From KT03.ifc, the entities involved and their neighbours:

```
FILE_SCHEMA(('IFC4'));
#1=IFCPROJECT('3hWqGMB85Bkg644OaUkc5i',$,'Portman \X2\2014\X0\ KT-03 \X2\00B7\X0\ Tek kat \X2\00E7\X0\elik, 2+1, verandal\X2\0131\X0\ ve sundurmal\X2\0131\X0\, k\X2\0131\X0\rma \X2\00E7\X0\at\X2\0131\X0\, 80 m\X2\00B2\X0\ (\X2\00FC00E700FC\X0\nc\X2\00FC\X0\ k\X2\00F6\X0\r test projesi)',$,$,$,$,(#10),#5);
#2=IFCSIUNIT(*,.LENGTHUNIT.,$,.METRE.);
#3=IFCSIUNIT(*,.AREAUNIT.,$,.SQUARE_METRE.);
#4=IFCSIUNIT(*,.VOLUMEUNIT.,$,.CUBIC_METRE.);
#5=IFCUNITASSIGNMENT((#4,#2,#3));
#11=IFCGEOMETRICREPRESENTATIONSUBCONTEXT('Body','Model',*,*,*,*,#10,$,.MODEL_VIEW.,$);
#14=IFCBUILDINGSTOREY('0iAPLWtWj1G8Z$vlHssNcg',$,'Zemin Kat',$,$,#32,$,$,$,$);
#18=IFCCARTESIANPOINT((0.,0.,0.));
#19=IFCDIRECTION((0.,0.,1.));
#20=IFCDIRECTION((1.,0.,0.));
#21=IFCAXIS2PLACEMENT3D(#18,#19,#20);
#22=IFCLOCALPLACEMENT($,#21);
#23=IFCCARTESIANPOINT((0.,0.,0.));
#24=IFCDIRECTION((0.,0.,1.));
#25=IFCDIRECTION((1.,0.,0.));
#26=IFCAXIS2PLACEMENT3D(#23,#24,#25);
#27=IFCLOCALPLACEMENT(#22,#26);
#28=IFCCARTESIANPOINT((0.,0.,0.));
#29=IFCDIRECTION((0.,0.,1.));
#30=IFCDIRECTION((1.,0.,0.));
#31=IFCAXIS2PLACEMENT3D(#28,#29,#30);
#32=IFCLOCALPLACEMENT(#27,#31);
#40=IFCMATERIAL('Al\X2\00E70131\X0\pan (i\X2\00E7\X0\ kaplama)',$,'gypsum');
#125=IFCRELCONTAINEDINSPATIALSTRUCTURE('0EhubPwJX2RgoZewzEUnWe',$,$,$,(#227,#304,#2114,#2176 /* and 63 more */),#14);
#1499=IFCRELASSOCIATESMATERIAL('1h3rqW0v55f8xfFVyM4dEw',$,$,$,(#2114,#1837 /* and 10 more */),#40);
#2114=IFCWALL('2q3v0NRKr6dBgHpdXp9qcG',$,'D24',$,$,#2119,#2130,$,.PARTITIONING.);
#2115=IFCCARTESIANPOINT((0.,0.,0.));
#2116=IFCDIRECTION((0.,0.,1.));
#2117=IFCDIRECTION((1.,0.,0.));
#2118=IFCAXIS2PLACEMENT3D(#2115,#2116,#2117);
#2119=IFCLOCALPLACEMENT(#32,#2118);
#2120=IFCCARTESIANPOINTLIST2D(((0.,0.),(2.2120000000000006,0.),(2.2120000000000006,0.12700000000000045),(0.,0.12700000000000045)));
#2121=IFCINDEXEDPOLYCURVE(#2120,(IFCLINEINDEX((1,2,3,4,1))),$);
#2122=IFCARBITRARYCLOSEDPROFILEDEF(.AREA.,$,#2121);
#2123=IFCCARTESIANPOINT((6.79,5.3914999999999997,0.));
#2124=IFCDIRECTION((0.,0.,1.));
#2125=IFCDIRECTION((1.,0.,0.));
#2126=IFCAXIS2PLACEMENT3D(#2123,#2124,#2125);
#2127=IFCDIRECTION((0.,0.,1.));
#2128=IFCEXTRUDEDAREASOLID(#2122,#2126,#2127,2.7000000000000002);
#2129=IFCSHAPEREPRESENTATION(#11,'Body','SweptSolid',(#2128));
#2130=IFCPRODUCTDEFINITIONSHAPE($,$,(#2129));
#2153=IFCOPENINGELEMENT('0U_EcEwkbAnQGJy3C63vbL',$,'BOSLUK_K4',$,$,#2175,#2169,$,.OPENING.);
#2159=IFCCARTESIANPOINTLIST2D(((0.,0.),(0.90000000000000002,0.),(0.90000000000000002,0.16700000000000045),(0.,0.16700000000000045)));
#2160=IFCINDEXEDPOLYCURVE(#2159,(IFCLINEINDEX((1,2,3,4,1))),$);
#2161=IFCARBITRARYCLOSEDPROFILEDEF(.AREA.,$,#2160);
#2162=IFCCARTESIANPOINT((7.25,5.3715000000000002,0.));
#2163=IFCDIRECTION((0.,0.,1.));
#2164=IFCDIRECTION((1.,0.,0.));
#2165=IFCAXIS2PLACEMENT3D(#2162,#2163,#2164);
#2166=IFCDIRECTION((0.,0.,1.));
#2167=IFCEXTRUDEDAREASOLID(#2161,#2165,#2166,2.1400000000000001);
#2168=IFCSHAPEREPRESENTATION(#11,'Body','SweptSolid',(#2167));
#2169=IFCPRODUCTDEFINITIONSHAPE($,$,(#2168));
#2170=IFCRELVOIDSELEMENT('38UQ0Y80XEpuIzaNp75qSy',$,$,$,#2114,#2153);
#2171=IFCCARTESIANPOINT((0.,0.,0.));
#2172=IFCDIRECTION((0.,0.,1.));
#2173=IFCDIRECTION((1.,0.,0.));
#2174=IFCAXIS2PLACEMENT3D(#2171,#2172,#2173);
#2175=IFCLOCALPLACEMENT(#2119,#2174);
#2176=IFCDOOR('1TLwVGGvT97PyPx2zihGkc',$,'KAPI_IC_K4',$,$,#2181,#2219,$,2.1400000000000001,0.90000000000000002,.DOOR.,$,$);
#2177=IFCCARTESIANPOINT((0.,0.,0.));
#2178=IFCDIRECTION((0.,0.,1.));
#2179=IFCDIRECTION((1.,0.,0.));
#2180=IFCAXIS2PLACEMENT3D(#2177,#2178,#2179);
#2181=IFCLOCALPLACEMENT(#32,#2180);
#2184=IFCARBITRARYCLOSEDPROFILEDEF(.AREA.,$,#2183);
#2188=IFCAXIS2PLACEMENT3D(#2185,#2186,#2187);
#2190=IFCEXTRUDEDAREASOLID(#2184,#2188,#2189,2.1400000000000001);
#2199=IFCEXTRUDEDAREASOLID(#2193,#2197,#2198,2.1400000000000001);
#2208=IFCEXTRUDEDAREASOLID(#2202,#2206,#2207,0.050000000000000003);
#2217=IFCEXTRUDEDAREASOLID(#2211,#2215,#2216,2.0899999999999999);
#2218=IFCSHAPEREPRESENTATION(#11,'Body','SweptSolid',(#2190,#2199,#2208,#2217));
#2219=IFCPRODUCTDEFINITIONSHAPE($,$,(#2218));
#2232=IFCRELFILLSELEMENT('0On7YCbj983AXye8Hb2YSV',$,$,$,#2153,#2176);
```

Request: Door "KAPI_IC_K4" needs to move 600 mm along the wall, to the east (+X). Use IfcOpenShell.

```python
import ifcopenshell
import ifcopenshell.api.geometry
import ifcopenshell.util.placement

model = ifcopenshell.open("KT03.ifc")

door = model.by_guid("1TLwVGGvT97PyPx2zihGkc")
opening = door.FillsVoids[0].RelatingOpeningElement
wall = opening.VoidsElements[0].RelatingBuildingElement

wall_matrix = ifcopenshell.util.placement.get_local_placement(wall.ObjectPlacement)
shift = wall_matrix[:3, 0] * 0.6
before = ifcopenshell.util.placement.get_local_placement(door.ObjectPlacement)[:3, 3].copy()

# The door is not placed relative to its opening, so move both.
for product in (opening, door):
    matrix = ifcopenshell.util.placement.get_local_placement(product.ObjectPlacement)
    matrix[:3, 3] += shift
    ifcopenshell.api.geometry.edit_object_placement(model, product=product, matrix=matrix, is_si=False)

after = ifcopenshell.util.placement.get_local_placement(door.ObjectPlacement)[:3, 3]
print("door moved by", (after - before).round(3) + 0.0)

model.write("KT03_edited.ifc")
```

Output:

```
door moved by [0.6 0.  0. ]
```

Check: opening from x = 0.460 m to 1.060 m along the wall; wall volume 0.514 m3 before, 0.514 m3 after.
